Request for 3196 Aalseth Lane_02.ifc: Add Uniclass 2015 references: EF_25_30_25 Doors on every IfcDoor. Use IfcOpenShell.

First a look at what the model holds.

```python
import ifcopenshell

model = ifcopenshell.open("3196 Aalseth Lane_02.ifc")
print(model.schema)
print("classifications:", [c.Name for c in model.by_type("IfcClassification")])
for ifc_class in ("IfcDoor", "IfcRoof", "IfcStair", "IfcWall", "IfcWindow"):
    print(ifc_class, len(model.by_type(ifc_class)))
```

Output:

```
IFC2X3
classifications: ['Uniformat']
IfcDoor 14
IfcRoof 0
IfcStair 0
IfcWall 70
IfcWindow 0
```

```python
import ifcopenshell
import ifcopenshell.api.classification

model = ifcopenshell.open("3196 Aalseth Lane_02.ifc")

# IFC2X3 requires Source and Edition and has no link from the project to the system.
system = model.create_entity("IfcClassification", Source="NBS", Edition="2015", Name="Uniclass 2015")

codes = {
    "IfcDoor": ("EF_25_30_25", "Doors"),
}
for ifc_class, (code, name) in codes.items():
    products = model.by_type(ifc_class)
    ifcopenshell.api.classification.add_reference(
        model, products=products, classification=system, identification=code, name=name
    )
    print(code, len(products))

model.write("3196 Aalseth Lane_02_updated.ifc")
```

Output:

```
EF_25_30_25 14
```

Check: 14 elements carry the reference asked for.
